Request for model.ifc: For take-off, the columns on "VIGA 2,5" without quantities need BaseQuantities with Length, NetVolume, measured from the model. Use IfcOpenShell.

First a look at what the model holds.

```python
import ifcopenshell
import ifcopenshell.util.element
import ifcopenshell.util.unit

model = ifcopenshell.open("model.ifc")
print(model.schema)
for unit_type in ("LENGTHUNIT", "AREAUNIT", "VOLUMEUNIT"):
    print(unit_type, ifcopenshell.util.unit.calculate_unit_scale(model, unit_type))
storey = next(s for s in model.by_type("IfcBuildingStorey") if s.Name == "VIGA 2,5")
columns = [e for e in ifcopenshell.util.element.get_decomposition(storey) if e.is_a("IfcColumn")]
for e in sorted(columns, key=lambda e: e.id()):
    print(e.id(), e.is_a(), e.Name, list(ifcopenshell.util.element.get_psets(e, qtos_only=True)), sep=" | ")
```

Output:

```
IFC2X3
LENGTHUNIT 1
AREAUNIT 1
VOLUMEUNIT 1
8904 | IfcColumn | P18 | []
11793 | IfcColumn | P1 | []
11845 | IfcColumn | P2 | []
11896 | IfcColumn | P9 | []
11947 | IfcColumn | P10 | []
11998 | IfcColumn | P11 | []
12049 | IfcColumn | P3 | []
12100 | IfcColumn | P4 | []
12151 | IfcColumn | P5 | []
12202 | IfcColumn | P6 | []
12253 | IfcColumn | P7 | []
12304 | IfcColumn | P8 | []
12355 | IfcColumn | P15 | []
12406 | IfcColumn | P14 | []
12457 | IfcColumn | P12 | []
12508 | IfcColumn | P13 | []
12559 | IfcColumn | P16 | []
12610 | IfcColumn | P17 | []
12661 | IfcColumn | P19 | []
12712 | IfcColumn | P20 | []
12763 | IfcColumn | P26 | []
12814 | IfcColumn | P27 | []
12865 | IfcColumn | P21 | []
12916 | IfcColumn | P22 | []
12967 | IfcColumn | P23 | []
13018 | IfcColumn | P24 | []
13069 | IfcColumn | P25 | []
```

```python
import ifcopenshell
import ifcopenshell.api.pset
import ifcopenshell.geom
import ifcopenshell.util.element
import ifcopenshell.util.shape
import ifcopenshell.util.unit

model = ifcopenshell.open("model.ifc")
unit_scale = ifcopenshell.util.unit.calculate_unit_scale(model)
volume_scale = ifcopenshell.util.unit.calculate_unit_scale(model, "VOLUMEUNIT")
settings = ifcopenshell.geom.settings()

storey = next(s for s in model.by_type("IfcBuildingStorey") if s.Name == "VIGA 2,5")
columns = [e for e in ifcopenshell.util.element.get_decomposition(storey) if e.is_a("IfcColumn")]

for e in sorted(columns, key=lambda e: e.id()):
    if ifcopenshell.util.element.get_psets(e, qtos_only=True, should_inherit=False):
        continue
    # Geometry comes back in metres, in the element's own axes.
    shape = ifcopenshell.geom.create_shape(settings, e)
    values = {
        "Length": ifcopenshell.util.shape.get_z(shape.geometry) / unit_scale,
        "NetVolume": ifcopenshell.util.shape.get_volume(shape.geometry) / volume_scale,
    }
    qto = ifcopenshell.api.pset.add_qto(model, product=e, name="BaseQuantities")
    ifcopenshell.api.pset.edit_qto(model, qto=qto, properties=values)
    print(e.id(), {k: round(v, 3) for k, v in values.items()})

model.write("model_rev.ifc")
```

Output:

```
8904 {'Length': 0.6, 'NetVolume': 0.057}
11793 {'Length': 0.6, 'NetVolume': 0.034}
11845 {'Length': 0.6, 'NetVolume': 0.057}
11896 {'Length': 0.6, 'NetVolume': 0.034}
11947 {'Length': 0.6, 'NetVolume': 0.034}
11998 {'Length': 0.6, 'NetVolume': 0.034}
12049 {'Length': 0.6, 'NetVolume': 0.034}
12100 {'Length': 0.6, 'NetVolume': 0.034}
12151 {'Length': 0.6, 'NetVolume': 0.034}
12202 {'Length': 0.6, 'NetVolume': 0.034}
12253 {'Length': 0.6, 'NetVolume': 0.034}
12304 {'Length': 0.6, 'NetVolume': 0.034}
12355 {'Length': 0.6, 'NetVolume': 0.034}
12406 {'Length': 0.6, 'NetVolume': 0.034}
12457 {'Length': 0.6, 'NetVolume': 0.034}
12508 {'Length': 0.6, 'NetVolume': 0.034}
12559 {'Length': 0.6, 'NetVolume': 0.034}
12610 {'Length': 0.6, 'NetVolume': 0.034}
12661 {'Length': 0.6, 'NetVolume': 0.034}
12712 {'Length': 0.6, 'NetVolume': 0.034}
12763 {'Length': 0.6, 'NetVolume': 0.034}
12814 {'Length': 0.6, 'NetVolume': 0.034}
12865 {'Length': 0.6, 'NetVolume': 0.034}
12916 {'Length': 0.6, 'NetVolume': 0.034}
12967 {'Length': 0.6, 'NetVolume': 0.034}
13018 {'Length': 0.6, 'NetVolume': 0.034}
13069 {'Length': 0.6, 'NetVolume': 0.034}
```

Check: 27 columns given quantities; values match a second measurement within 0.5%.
